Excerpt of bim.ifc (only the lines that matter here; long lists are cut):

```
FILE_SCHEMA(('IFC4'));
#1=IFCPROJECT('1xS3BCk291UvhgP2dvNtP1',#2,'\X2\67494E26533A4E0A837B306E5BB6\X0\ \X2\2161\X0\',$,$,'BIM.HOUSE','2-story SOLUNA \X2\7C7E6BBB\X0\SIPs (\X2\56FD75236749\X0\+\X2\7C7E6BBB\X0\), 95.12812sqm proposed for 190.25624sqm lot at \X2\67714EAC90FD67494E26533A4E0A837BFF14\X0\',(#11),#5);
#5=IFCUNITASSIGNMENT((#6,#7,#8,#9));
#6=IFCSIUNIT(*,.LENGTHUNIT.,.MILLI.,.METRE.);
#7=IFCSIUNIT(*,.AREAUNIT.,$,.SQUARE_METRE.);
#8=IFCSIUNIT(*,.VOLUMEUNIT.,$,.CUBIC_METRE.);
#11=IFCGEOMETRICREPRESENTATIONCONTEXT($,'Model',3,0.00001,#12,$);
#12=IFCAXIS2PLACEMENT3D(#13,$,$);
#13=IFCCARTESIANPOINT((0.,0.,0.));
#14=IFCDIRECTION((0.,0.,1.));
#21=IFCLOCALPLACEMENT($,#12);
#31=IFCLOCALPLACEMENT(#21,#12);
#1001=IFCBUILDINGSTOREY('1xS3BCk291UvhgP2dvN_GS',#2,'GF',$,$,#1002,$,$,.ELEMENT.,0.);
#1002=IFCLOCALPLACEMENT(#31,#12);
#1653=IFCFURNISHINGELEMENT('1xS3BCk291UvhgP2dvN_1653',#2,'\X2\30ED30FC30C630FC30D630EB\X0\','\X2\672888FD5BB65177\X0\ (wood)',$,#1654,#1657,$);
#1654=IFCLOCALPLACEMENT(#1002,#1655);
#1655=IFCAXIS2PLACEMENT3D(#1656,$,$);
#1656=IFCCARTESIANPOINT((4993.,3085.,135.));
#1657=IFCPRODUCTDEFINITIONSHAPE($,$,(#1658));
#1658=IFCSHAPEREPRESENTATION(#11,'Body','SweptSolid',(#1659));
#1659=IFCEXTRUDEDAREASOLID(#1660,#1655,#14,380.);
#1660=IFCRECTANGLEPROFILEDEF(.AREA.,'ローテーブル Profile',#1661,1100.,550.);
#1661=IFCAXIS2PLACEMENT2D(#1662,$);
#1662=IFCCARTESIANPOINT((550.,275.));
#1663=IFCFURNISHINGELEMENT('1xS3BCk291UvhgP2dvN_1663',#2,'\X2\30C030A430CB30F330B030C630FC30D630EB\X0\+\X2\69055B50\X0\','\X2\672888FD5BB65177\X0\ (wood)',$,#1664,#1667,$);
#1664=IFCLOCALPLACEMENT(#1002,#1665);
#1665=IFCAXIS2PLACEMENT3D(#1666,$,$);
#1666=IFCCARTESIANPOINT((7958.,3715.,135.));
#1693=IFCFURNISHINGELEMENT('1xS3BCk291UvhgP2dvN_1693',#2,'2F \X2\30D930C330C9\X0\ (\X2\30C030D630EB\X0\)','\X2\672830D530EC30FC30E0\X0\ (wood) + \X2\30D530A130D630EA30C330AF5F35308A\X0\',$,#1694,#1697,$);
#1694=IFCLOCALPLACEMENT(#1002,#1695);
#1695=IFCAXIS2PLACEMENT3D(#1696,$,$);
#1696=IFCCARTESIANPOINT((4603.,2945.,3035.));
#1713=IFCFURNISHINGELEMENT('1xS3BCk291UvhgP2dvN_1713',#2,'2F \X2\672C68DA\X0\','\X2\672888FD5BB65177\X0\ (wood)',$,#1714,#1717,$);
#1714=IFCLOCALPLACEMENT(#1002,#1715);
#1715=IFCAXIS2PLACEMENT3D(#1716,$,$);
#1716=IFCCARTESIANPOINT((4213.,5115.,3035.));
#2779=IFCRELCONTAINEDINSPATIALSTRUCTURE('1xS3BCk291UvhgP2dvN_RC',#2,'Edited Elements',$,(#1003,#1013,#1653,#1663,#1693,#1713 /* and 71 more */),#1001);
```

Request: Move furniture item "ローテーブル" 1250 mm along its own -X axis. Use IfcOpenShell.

```python
import ifcopenshell
import ifcopenshell.api.geometry
import ifcopenshell.util.placement
import ifcopenshell.util.unit

model = ifcopenshell.open("bim.ifc")
unit_scale = ifcopenshell.util.unit.calculate_unit_scale(model)

item = model.by_guid("1xS3BCk291UvhgP2dvN_1653")
matrix = ifcopenshell.util.placement.get_local_placement(item.ObjectPlacement)
matrix[:3, 3] -= matrix[:3, 0] * 1.25 / unit_scale
ifcopenshell.api.geometry.edit_object_placement(model, product=item, matrix=matrix, is_si=False)

print(ifcopenshell.util.placement.get_local_placement(item.ObjectPlacement).round(3) + 0.0)

model.write("bim-out.ifc")
```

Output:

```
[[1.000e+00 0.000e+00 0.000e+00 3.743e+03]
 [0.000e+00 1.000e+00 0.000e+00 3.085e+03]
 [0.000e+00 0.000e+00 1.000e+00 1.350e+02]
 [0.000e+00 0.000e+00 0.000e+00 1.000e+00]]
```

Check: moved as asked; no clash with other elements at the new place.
